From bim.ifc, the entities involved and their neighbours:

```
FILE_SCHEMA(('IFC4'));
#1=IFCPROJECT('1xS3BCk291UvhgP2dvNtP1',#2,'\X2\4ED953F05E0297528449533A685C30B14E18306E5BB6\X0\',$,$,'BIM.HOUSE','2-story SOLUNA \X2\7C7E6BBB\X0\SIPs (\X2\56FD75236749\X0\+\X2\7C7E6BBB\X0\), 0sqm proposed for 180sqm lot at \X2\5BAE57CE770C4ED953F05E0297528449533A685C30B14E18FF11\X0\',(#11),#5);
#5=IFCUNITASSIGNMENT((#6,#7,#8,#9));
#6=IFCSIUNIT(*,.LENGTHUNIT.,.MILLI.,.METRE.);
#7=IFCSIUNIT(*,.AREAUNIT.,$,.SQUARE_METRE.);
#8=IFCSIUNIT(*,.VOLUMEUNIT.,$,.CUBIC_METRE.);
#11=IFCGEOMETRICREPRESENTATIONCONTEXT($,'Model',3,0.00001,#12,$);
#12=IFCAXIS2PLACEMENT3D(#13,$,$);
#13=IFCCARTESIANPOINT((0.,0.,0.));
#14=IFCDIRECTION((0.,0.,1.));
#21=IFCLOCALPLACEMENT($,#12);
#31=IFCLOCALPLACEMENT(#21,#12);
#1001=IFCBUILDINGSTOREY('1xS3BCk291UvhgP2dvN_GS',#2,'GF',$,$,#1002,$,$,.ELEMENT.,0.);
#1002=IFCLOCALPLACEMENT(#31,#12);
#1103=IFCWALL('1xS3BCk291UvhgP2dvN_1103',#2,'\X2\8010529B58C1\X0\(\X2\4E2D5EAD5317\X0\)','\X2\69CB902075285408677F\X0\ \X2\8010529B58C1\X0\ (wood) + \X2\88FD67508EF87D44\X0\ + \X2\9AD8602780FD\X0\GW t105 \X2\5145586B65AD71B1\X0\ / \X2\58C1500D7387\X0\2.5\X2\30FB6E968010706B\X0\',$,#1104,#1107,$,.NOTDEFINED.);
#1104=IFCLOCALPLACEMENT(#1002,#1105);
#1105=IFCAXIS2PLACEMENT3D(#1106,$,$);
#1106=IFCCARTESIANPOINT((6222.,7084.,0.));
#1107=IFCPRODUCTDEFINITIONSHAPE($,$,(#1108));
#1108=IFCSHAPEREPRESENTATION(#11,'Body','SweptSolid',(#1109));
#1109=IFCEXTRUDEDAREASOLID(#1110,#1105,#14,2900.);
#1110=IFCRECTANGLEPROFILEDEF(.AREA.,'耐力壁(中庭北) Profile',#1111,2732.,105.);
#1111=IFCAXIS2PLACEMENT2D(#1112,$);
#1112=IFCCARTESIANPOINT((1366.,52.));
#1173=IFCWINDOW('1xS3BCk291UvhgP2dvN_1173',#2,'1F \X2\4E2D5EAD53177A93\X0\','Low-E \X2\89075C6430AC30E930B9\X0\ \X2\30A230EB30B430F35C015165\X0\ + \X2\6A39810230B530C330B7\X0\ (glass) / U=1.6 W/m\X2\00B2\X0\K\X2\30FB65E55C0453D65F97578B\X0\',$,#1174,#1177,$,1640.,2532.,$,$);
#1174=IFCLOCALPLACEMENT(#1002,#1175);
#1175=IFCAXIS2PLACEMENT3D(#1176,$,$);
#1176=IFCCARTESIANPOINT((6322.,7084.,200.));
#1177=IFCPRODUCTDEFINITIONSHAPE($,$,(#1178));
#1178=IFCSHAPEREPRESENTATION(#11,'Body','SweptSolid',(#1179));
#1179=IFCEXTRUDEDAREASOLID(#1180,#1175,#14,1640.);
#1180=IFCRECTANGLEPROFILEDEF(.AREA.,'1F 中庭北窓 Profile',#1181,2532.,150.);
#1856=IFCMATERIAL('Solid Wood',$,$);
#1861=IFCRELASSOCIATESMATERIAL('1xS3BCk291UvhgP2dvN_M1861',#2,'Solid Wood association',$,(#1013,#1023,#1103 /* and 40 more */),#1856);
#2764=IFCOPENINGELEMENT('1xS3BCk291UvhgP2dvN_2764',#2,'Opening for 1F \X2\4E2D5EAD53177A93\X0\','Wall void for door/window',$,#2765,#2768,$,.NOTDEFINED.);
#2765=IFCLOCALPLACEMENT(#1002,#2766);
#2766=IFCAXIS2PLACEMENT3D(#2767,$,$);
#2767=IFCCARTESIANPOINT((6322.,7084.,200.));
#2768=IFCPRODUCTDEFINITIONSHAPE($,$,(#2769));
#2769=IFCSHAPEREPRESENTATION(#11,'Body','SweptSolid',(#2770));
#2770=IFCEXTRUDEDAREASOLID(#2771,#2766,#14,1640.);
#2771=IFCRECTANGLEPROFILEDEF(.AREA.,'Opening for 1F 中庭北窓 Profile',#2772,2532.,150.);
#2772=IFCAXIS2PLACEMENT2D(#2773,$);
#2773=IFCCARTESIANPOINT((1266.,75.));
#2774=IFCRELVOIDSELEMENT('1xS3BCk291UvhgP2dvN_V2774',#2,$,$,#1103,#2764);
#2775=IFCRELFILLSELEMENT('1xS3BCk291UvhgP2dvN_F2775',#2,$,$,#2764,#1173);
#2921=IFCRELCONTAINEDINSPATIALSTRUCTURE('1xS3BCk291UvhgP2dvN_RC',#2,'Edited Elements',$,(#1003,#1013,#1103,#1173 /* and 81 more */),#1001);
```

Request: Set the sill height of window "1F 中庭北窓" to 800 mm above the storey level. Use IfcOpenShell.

```python
import numpy as np
import ifcopenshell
import ifcopenshell.api.geometry
import ifcopenshell.geom
import ifcopenshell.util.element
import ifcopenshell.util.placement
import ifcopenshell.util.shape
import ifcopenshell.util.unit

model = ifcopenshell.open("bim.ifc")
unit_scale = ifcopenshell.util.unit.calculate_unit_scale(model)

window = model.by_guid("1xS3BCk291UvhgP2dvN_1173")
opening = window.FillsVoids[0].RelatingOpeningElement
storey = ifcopenshell.util.element.get_container(window, ifc_class="IfcBuildingStorey")
level = ifcopenshell.util.placement.get_local_placement(storey.ObjectPlacement)[2, 3]

# The opening's origin need not be at the sill, so measure its lowest point.
shape = ifcopenshell.geom.create_shape(ifcopenshell.geom.settings(), opening)
bottom = ifcopenshell.util.shape.get_shape_bottom_elevation(shape, shape.geometry) / unit_scale
dz = level + 800.0 - bottom

shift = np.array([0.0, 0.0, dz])
# The window is not placed relative to its opening, so move both.
for product in (opening, window):
    matrix = ifcopenshell.util.placement.get_local_placement(product.ObjectPlacement)
    matrix[:3, 3] += shift
    ifcopenshell.api.geometry.edit_object_placement(model, product=product, matrix=matrix, is_si=False)

print(f"moved by {dz * unit_scale:+.3f} m")

model.write("bim_edited.ifc")
```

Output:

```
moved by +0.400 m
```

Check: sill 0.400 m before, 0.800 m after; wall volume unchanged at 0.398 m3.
